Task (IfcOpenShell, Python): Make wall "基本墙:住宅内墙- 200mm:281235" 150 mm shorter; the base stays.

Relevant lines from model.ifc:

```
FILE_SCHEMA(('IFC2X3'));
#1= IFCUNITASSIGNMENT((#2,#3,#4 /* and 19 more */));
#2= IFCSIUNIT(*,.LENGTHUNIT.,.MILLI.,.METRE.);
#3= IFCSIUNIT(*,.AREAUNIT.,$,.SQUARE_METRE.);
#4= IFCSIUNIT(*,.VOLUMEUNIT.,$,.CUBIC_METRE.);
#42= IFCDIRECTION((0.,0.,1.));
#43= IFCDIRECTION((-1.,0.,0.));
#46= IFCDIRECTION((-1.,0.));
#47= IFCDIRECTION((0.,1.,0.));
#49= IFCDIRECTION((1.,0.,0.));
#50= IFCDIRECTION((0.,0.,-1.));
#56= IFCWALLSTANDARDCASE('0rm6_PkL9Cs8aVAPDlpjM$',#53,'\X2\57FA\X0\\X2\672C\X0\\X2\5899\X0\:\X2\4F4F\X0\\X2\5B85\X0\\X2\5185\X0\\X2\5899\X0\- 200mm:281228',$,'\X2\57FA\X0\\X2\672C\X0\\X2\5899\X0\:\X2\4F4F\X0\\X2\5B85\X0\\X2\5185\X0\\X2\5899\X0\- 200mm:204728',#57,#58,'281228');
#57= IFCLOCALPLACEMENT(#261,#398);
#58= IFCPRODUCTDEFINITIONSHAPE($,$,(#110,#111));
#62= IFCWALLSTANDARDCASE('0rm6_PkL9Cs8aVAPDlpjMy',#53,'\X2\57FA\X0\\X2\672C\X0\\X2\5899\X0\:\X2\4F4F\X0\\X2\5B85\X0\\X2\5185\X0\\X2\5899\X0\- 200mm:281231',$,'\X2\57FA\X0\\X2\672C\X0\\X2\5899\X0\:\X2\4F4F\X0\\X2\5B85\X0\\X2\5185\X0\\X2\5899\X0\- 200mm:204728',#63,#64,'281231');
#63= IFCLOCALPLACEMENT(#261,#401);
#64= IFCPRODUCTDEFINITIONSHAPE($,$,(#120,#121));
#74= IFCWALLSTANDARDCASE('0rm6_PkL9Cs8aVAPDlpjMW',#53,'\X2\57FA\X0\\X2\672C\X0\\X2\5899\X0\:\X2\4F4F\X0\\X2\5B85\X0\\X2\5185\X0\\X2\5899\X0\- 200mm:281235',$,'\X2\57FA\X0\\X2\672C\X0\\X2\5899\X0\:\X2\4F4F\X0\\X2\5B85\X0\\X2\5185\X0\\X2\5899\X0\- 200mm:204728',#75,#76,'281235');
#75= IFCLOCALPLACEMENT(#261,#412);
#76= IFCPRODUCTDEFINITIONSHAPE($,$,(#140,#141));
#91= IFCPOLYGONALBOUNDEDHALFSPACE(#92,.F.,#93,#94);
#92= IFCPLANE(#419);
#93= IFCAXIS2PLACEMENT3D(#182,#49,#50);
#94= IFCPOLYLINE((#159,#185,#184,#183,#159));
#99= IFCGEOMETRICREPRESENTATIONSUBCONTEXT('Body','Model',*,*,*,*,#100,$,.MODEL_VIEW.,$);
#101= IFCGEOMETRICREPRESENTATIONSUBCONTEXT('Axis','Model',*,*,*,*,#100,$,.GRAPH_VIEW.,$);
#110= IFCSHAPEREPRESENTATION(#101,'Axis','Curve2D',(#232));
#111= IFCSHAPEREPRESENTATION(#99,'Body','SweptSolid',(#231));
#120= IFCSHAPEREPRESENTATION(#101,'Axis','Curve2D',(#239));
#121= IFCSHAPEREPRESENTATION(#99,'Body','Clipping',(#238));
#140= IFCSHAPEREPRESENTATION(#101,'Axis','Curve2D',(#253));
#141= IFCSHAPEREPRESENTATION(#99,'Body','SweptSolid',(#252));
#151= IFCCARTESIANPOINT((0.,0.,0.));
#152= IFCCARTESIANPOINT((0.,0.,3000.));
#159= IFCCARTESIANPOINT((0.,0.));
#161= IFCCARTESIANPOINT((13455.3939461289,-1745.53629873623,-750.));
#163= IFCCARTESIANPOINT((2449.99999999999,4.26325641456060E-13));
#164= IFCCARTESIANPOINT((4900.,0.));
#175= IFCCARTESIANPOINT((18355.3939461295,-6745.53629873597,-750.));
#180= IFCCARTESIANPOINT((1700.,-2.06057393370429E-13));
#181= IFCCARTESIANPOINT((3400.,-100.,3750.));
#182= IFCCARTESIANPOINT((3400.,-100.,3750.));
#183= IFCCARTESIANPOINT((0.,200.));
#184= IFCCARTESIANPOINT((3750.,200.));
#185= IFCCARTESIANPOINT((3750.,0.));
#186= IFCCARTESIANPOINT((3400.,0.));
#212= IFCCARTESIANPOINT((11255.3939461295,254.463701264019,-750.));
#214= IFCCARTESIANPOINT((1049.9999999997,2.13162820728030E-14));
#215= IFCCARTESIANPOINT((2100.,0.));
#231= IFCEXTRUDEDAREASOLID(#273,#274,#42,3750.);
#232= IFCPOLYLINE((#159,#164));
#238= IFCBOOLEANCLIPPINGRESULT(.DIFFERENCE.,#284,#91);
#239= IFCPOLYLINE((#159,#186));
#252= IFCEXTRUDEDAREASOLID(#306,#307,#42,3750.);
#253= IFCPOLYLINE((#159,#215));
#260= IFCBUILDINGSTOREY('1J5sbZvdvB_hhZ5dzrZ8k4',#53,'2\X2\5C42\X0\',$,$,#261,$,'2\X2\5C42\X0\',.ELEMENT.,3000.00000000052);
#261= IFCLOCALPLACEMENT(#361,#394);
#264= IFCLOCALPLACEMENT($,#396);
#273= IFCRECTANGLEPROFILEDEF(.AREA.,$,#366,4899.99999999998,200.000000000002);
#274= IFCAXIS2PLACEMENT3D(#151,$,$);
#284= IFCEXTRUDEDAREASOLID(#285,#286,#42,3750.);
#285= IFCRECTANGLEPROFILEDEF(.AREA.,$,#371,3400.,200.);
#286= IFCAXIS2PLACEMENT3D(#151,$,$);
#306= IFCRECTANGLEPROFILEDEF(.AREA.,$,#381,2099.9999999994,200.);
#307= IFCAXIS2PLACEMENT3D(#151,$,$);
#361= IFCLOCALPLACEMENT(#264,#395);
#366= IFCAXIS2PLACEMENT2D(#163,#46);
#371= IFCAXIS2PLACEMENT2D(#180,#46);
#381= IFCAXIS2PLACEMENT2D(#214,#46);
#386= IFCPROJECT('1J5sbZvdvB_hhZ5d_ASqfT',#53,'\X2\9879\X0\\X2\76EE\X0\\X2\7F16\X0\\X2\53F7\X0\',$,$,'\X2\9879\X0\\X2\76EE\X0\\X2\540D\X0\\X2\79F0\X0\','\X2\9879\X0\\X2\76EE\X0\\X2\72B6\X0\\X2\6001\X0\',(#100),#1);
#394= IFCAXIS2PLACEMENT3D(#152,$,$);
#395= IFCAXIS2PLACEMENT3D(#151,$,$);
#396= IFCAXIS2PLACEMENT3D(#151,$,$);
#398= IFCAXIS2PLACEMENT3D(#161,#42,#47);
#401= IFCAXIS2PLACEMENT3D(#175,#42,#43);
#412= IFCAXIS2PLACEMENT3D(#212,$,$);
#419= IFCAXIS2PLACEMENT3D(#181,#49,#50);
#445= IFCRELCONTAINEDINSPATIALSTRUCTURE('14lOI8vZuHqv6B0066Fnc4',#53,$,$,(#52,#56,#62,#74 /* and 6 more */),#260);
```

```python
import ifcopenshell
import ifcopenshell.geom
import ifcopenshell.util.representation
import ifcopenshell.util.shape

model = ifcopenshell.open("model.ifc")
settings = ifcopenshell.geom.settings()


def volume(element):
    """Net volume in cubic metres, openings subtracted."""
    shape = ifcopenshell.geom.create_shape(settings, element)
    return ifcopenshell.util.shape.get_volume(shape.geometry)


wall = model.by_guid("0rm6_PkL9Cs8aVAPDlpjMW")
before = volume(wall)

body = ifcopenshell.util.representation.get_representation(wall, "Model", "Body")
solid = body.Items[0]
old_height = solid.Depth
solid.Depth -= 150.0
after = volume(wall)

print(f"height {old_height:g} -> {solid.Depth:g}, volume {before:.3f} -> {after:.3f} m3")

model.write("model_rev.ifc")
```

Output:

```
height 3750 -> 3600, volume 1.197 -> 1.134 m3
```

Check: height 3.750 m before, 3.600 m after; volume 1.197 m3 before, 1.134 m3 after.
